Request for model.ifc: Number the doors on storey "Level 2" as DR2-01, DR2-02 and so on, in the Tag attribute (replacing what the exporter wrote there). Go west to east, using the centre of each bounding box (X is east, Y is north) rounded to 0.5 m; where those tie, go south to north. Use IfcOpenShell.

First a look at what the model holds.

```python
import ifcopenshell
import ifcopenshell.util.element
import ifcopenshell.util.placement

model = ifcopenshell.open("model.ifc")
print(model.schema)
storey = next(s for s in model.by_type("IfcBuildingStorey") if s.Name == "Level 2")
doors = [e for e in ifcopenshell.util.element.get_decomposition(storey) if e.is_a("IfcDoor")]
for e in sorted(doors, key=lambda e: e.id()):
    origin = ifcopenshell.util.placement.get_local_placement(e.ObjectPlacement)[:3, 3]
    print(e.id(), e.Tag, e.Name, origin.round(2) + 0.0, sep=" | ")
```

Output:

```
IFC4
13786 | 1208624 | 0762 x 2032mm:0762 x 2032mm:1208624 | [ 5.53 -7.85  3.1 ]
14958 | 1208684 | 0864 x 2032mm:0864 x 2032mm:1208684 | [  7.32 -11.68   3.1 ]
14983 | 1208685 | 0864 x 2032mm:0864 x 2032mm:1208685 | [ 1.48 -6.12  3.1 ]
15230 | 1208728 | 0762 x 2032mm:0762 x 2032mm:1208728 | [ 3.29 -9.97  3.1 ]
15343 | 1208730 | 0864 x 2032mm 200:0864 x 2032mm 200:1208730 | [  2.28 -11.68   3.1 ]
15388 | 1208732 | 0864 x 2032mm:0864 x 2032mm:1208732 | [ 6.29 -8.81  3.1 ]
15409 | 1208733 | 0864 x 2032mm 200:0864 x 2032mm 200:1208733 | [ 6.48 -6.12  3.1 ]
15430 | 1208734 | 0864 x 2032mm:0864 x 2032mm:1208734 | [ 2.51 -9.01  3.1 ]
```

```python
import ifcopenshell
import ifcopenshell.geom
import ifcopenshell.util.element
import ifcopenshell.util.shape

model = ifcopenshell.open("model.ifc")
settings = ifcopenshell.geom.settings()
settings.set("use-world-coords", True)


def centre(element):
    shape = ifcopenshell.geom.create_shape(settings, element)
    return ifcopenshell.util.shape.get_bbox_centroid(shape.geometry)


storey = next(s for s in model.by_type("IfcBuildingStorey") if s.Name == "Level 2")
doors = [e for e in ifcopenshell.util.element.get_decomposition(storey) if e.is_a("IfcDoor")]

# Insertion points can sit at a corner or the storey origin, so sort by the geometry (in metres).
centres = {e: centre(e) for e in doors}
doors.sort(key=lambda e: (round(centres[e][0] / 0.5), centres[e][1]))

for i, e in enumerate(doors, start=1):
    number = f"DR2-{i:02d}"
    e.Tag = number
    print(e.id(), number)

model.write("model_rev.ifc")
```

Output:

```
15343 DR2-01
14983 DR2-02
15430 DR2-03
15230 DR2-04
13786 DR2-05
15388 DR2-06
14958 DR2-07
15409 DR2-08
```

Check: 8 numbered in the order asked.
